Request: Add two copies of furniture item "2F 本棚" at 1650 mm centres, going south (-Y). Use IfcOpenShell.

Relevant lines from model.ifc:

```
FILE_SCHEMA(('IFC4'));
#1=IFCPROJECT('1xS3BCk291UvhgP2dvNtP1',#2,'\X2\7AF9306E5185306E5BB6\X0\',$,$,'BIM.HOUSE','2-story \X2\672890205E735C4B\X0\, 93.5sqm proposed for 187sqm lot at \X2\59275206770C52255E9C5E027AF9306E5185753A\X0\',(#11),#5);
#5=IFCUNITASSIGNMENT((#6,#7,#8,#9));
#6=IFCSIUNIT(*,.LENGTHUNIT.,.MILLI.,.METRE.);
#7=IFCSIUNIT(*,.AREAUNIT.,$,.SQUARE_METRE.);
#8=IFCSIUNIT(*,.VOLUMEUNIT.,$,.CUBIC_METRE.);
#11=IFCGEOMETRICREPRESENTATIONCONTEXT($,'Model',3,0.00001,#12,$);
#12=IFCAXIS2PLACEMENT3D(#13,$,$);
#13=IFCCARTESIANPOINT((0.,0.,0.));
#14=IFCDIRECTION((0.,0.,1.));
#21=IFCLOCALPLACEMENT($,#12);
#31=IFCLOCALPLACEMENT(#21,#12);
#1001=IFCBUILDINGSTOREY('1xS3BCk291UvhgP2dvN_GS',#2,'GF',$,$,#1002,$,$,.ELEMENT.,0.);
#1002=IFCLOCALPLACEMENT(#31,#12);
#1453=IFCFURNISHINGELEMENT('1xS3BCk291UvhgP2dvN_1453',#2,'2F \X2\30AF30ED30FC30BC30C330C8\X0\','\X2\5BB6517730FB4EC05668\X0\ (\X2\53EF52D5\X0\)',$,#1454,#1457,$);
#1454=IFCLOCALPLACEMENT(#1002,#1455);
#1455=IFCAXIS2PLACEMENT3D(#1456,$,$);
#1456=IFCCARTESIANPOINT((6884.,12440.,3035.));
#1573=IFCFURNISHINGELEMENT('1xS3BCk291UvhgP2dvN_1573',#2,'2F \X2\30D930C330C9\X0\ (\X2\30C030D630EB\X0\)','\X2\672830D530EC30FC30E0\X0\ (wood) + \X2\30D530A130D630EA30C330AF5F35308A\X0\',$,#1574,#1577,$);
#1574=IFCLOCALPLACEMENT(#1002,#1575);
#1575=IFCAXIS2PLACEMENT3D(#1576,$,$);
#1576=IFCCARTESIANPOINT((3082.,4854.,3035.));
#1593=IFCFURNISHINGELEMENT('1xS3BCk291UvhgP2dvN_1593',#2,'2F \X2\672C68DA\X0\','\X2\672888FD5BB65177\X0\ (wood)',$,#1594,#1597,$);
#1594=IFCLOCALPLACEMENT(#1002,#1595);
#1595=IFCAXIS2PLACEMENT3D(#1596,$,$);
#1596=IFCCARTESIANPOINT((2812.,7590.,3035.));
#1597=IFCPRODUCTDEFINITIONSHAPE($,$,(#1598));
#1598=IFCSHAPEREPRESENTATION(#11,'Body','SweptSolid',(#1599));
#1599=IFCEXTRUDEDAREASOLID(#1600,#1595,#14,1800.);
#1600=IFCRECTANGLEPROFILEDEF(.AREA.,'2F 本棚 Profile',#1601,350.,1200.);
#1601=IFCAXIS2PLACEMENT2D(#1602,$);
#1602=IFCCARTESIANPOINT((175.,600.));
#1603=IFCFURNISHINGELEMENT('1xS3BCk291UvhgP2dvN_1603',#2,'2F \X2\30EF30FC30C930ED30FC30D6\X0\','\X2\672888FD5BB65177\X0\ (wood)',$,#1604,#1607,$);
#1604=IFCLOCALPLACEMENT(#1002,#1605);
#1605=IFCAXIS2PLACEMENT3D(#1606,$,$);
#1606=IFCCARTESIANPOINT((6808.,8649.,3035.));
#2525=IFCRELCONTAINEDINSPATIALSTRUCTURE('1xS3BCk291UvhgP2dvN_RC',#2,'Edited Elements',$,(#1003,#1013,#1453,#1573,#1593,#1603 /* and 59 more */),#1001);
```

```python
import numpy as np
import ifcopenshell
import ifcopenshell.api.geometry
import ifcopenshell.api.root
import ifcopenshell.util.element
import ifcopenshell.util.placement

model = ifcopenshell.open("model.ifc")


def reuse_history(source, copy):
    """copy_class also copies each property set's owner history, people and application; keep the originals."""
    for rel in copy.IsDefinedBy:
        if rel.is_a("IfcRelDefinesByProperties") and (history := rel.RelatingPropertyDefinition.OwnerHistory):
            rel.RelatingPropertyDefinition.OwnerHistory = source.OwnerHistory
            ifcopenshell.util.element.remove_deep2(model, history)


source = model.by_guid("1xS3BCk291UvhgP2dvN_1593")
base = ifcopenshell.util.placement.get_local_placement(source.ObjectPlacement)
step = np.array([0.0, -1.0, 0.0]) * 1650.0

for i in range(1, 3):
    copy = ifcopenshell.api.root.copy_class(model, product=source)
    copy.Representation = ifcopenshell.util.element.copy_deep(
        model, source.Representation, exclude=["IfcGeometricRepresentationContext", "IfcRepresentationMap"]
    )
    reuse_history(source, copy)
    matrix = base.copy()
    matrix[:3, 3] += i * step
    print("added at", matrix[:3, 3].round(3) + 0.0)
    ifcopenshell.api.geometry.edit_object_placement(model, product=copy, matrix=matrix, is_si=False)

model.write("model_edited.ifc")
```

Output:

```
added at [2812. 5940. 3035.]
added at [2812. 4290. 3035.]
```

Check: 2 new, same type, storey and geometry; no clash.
